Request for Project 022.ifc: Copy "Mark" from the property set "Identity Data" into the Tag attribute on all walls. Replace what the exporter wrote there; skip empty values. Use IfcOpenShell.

First a look at what the model holds.

```python
import ifcopenshell
import ifcopenshell.util.element

model = ifcopenshell.open("Project 022.ifc")
print(model.schema)
walls = model.by_type("IfcWall")
print(len(walls), "walls")
for e in walls[:8]:
    source = ifcopenshell.util.element.get_pset(e, "Identity Data", "Mark")
    target = e.Tag
    print(e.id(), repr(source), repr(target), sep=" | ")
```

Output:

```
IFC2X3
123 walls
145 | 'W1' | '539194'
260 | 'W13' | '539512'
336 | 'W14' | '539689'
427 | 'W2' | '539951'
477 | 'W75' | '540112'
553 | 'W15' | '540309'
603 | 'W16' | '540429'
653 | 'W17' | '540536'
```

```python
import ifcopenshell
import ifcopenshell.util.element

model = ifcopenshell.open("Project 022.ifc")

count = 0
for e in model.by_type("IfcWall"):
    value = ifcopenshell.util.element.get_pset(e, "Identity Data", "Mark")
    current = e.Tag
    if not value or not value.strip() or current == value:
        continue
    e.Tag = value
    count += 1

print(count, "walls updated")

model.write("Project 022-out.ifc")
```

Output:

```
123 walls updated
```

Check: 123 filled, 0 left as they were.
